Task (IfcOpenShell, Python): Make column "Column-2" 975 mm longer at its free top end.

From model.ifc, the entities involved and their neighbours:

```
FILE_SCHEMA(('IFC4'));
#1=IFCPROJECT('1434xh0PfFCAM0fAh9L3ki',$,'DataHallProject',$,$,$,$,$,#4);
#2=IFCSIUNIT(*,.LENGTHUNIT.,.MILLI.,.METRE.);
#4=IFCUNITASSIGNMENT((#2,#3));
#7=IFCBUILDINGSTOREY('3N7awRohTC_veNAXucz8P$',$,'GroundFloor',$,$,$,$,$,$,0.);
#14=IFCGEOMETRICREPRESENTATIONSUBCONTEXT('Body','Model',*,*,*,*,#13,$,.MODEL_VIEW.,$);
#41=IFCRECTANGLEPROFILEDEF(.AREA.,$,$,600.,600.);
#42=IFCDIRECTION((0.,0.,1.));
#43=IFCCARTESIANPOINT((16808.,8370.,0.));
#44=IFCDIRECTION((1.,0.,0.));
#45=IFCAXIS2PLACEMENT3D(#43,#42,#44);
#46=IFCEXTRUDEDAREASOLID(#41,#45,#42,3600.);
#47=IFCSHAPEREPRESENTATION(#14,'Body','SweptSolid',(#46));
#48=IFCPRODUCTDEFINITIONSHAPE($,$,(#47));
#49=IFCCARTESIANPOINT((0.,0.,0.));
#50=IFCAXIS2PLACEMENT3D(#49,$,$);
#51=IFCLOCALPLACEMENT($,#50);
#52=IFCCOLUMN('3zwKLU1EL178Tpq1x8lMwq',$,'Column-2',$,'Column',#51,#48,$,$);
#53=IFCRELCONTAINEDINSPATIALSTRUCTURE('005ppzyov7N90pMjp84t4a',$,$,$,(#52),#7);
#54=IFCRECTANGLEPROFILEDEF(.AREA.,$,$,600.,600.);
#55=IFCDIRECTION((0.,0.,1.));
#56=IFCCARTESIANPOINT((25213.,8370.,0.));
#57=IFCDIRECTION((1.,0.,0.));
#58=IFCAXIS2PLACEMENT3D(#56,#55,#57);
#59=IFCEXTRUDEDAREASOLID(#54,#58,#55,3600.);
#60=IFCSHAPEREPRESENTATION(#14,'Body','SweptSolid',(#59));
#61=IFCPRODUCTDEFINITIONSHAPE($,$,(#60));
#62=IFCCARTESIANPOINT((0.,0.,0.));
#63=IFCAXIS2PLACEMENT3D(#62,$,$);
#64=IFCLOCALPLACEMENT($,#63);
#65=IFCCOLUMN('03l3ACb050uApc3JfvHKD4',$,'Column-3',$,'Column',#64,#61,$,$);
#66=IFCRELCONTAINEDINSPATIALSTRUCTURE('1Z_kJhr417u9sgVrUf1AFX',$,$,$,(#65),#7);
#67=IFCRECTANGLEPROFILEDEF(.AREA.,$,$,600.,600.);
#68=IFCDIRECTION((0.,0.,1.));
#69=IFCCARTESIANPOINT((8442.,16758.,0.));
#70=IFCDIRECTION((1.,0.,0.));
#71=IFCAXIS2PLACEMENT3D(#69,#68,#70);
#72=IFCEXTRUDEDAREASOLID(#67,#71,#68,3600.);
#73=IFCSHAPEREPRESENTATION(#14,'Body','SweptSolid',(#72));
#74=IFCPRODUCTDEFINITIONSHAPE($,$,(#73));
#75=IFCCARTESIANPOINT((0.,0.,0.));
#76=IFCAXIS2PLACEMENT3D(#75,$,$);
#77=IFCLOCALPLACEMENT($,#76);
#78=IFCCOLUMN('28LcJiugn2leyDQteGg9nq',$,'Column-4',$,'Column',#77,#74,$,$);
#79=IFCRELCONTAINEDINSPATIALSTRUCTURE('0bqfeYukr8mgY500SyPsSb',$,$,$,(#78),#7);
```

```python
import ifcopenshell
import ifcopenshell.util.representation
import ifcopenshell.util.unit

model = ifcopenshell.open("model.ifc")
unit_scale = ifcopenshell.util.unit.calculate_unit_scale(model)

member = model.by_id(52)
change = 0.975 / unit_scale

# The extrusion runs towards the end named, so only its depth changes.
body = ifcopenshell.util.representation.get_representation(member, "Model", "Body")
solid = body.Items[0]
old_length = solid.Depth
solid.Depth += change

print(f"length {old_length:g} -> {solid.Depth:g}")

model.write("model_rev.ifc")
```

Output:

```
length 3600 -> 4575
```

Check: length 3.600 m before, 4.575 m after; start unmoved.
